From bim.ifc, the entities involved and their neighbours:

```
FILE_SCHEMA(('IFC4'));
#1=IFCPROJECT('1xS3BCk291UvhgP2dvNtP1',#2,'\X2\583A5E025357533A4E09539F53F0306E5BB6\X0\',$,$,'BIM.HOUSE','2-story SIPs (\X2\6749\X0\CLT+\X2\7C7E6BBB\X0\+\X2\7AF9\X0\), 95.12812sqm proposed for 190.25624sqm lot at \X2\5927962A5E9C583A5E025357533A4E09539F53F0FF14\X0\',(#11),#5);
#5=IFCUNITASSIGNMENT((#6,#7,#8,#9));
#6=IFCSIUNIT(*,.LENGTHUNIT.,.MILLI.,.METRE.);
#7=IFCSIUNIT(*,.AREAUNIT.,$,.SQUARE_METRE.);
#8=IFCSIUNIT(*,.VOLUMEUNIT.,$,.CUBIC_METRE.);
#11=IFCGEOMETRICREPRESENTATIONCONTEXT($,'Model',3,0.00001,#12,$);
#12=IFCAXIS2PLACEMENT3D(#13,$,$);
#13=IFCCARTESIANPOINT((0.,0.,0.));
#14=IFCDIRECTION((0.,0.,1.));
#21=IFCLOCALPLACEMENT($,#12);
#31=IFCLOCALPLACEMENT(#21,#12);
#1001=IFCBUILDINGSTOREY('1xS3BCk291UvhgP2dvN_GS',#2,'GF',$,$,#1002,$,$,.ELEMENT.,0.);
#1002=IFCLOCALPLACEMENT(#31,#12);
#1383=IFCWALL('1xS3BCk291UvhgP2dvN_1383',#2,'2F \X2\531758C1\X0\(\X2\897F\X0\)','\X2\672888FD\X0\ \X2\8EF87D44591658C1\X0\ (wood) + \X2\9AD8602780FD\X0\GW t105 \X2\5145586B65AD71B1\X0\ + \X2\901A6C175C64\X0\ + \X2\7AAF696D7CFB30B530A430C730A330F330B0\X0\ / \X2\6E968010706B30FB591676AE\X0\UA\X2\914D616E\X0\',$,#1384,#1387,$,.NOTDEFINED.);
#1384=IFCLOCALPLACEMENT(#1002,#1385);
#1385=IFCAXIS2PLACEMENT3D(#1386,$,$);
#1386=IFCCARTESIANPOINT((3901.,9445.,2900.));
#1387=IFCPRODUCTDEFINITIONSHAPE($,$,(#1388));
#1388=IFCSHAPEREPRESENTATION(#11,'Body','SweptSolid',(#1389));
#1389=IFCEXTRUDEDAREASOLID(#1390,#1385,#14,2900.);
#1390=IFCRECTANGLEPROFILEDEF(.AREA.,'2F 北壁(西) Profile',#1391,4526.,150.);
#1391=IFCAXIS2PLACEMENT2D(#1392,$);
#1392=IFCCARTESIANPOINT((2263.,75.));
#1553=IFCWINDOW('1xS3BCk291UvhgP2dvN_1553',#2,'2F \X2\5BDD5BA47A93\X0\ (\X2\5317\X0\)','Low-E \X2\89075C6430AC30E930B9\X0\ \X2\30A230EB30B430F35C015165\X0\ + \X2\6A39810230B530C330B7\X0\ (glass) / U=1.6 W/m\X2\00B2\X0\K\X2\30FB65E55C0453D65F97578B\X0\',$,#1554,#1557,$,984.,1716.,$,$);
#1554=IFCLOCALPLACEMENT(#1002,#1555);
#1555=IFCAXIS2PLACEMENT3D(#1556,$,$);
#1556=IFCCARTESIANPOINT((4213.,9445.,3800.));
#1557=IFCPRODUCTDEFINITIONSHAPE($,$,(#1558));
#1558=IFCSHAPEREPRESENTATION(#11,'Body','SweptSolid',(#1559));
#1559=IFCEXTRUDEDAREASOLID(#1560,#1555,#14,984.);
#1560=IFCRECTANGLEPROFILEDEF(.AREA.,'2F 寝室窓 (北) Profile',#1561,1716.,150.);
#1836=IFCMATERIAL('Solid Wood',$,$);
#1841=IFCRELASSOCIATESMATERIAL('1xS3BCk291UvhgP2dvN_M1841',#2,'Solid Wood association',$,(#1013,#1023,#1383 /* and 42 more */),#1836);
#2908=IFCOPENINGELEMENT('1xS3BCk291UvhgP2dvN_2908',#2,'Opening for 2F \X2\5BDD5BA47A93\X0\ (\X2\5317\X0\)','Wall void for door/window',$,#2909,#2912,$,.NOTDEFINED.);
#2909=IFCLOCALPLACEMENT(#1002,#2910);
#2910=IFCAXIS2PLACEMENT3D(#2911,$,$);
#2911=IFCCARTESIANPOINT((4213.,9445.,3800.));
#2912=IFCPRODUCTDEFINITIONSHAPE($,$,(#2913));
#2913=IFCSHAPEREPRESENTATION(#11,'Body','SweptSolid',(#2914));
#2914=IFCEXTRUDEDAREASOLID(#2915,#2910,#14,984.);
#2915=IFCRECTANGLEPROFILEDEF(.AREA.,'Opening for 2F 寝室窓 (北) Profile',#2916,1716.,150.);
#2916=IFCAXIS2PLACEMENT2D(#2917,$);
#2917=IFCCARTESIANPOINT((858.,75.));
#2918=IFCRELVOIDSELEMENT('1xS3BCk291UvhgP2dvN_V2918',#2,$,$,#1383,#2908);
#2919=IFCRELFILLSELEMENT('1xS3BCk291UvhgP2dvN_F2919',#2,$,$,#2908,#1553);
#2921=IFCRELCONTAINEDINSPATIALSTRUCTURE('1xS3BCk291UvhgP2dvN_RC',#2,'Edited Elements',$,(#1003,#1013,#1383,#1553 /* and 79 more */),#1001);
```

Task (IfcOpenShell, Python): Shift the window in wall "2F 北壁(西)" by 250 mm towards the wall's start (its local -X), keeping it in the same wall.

```python
import ifcopenshell
import ifcopenshell.api.geometry
import ifcopenshell.util.placement

model = ifcopenshell.open("bim.ifc")

window = model.by_guid("1xS3BCk291UvhgP2dvN_1553")
opening = window.FillsVoids[0].RelatingOpeningElement
wall = opening.VoidsElements[0].RelatingBuildingElement

wall_matrix = ifcopenshell.util.placement.get_local_placement(wall.ObjectPlacement)
shift = wall_matrix[:3, 0] * -250.0
before = ifcopenshell.util.placement.get_local_placement(window.ObjectPlacement)[:3, 3].copy()

# The window is not placed relative to its opening, so move both.
for product in (opening, window):
    matrix = ifcopenshell.util.placement.get_local_placement(product.ObjectPlacement)
    matrix[:3, 3] += shift
    ifcopenshell.api.geometry.edit_object_placement(model, product=product, matrix=matrix, is_si=False)

after = ifcopenshell.util.placement.get_local_placement(window.ObjectPlacement)[:3, 3]
print("window moved by", (after - before).round(3) + 0.0)

model.write("bim_rev.ifc")
```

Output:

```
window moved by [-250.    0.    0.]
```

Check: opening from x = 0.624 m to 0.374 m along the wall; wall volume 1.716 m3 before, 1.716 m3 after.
